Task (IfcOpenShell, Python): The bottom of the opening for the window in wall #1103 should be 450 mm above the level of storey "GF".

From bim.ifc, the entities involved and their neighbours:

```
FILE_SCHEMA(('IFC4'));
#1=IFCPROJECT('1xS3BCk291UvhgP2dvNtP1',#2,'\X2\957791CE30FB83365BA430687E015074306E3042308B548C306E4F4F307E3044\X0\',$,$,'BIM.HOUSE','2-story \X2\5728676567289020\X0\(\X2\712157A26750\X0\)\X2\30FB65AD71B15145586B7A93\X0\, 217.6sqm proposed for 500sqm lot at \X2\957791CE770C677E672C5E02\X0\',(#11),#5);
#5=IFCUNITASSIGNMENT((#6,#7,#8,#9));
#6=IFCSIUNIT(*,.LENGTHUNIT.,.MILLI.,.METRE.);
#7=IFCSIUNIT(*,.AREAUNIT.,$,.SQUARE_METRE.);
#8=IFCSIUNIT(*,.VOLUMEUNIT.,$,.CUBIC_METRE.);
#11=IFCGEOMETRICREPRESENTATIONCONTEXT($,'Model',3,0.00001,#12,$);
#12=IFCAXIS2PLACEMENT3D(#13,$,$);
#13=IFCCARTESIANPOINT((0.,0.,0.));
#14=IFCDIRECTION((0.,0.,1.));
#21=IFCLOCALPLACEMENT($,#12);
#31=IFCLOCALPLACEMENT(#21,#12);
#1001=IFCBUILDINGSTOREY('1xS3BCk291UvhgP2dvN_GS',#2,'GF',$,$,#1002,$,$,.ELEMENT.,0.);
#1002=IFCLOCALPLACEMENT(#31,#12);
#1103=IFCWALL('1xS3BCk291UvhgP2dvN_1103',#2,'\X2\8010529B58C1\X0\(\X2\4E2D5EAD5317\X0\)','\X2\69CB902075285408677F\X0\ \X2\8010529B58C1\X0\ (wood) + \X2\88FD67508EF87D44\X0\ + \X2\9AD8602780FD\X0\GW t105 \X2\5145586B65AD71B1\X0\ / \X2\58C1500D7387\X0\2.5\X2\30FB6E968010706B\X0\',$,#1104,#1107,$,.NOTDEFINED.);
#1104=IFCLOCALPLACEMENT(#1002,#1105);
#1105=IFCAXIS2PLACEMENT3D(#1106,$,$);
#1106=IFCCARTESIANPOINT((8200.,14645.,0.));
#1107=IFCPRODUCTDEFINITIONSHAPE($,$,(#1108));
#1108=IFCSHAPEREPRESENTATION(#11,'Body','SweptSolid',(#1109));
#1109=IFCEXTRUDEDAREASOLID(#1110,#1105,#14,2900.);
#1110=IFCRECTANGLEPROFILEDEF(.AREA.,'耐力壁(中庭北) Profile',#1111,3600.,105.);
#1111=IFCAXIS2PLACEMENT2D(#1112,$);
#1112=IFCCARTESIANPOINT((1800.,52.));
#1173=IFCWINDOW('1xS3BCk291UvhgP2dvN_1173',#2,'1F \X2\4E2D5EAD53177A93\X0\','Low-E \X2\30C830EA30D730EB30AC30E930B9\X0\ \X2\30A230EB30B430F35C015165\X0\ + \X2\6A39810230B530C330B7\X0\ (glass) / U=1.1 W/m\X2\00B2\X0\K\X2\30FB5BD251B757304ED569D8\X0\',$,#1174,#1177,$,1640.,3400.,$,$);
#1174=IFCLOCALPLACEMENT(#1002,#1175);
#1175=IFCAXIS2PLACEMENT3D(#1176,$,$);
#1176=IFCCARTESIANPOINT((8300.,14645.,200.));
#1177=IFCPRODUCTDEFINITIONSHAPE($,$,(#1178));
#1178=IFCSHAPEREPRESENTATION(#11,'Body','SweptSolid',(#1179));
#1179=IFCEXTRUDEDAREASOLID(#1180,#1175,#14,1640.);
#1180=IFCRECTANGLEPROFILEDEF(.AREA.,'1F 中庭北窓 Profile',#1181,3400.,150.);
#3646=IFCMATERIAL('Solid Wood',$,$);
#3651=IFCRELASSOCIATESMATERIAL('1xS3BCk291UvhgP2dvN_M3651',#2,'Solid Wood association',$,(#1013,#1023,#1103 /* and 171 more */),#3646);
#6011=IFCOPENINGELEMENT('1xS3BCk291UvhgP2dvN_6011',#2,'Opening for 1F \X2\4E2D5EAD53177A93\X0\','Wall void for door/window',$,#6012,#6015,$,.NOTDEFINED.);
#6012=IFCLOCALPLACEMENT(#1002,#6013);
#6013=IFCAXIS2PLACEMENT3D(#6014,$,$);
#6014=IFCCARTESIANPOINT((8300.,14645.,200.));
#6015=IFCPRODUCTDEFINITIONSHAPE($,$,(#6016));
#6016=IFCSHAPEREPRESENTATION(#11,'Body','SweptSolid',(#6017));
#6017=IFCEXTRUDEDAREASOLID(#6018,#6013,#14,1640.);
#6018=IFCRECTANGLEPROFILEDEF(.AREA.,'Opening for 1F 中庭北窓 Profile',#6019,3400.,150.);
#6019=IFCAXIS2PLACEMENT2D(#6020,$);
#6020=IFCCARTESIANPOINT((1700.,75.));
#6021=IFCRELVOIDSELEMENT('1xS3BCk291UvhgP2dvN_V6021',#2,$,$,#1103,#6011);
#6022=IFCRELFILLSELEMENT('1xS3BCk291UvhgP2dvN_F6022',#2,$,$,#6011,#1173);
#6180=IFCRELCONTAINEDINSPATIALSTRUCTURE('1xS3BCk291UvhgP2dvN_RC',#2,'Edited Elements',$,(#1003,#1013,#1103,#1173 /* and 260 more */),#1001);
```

```python
import numpy as np
import ifcopenshell
import ifcopenshell.api.geometry
import ifcopenshell.geom
import ifcopenshell.util.element
import ifcopenshell.util.placement
import ifcopenshell.util.shape
import ifcopenshell.util.unit

model = ifcopenshell.open("bim.ifc")
unit_scale = ifcopenshell.util.unit.calculate_unit_scale(model)

window = model.by_guid("1xS3BCk291UvhgP2dvN_1173")
opening = window.FillsVoids[0].RelatingOpeningElement
storey = ifcopenshell.util.element.get_container(window, ifc_class="IfcBuildingStorey")
level = ifcopenshell.util.placement.get_local_placement(storey.ObjectPlacement)[2, 3]

# The opening's origin need not be at the sill, so measure its lowest point.
shape = ifcopenshell.geom.create_shape(ifcopenshell.geom.settings(), opening)
bottom = ifcopenshell.util.shape.get_shape_bottom_elevation(shape, shape.geometry) / unit_scale
dz = level + 0.45 / unit_scale - bottom

shift = np.array([0.0, 0.0, dz])
# The window is not placed relative to its opening, so move both.
for product in (opening, window):
    matrix = ifcopenshell.util.placement.get_local_placement(product.ObjectPlacement)
    matrix[:3, 3] += shift
    ifcopenshell.api.geometry.edit_object_placement(model, product=product, matrix=matrix, is_si=False)

print(f"moved by {dz * unit_scale:+.3f} m")

model.write("bim-out.ifc")
```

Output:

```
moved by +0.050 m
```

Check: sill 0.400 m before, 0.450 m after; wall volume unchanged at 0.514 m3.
